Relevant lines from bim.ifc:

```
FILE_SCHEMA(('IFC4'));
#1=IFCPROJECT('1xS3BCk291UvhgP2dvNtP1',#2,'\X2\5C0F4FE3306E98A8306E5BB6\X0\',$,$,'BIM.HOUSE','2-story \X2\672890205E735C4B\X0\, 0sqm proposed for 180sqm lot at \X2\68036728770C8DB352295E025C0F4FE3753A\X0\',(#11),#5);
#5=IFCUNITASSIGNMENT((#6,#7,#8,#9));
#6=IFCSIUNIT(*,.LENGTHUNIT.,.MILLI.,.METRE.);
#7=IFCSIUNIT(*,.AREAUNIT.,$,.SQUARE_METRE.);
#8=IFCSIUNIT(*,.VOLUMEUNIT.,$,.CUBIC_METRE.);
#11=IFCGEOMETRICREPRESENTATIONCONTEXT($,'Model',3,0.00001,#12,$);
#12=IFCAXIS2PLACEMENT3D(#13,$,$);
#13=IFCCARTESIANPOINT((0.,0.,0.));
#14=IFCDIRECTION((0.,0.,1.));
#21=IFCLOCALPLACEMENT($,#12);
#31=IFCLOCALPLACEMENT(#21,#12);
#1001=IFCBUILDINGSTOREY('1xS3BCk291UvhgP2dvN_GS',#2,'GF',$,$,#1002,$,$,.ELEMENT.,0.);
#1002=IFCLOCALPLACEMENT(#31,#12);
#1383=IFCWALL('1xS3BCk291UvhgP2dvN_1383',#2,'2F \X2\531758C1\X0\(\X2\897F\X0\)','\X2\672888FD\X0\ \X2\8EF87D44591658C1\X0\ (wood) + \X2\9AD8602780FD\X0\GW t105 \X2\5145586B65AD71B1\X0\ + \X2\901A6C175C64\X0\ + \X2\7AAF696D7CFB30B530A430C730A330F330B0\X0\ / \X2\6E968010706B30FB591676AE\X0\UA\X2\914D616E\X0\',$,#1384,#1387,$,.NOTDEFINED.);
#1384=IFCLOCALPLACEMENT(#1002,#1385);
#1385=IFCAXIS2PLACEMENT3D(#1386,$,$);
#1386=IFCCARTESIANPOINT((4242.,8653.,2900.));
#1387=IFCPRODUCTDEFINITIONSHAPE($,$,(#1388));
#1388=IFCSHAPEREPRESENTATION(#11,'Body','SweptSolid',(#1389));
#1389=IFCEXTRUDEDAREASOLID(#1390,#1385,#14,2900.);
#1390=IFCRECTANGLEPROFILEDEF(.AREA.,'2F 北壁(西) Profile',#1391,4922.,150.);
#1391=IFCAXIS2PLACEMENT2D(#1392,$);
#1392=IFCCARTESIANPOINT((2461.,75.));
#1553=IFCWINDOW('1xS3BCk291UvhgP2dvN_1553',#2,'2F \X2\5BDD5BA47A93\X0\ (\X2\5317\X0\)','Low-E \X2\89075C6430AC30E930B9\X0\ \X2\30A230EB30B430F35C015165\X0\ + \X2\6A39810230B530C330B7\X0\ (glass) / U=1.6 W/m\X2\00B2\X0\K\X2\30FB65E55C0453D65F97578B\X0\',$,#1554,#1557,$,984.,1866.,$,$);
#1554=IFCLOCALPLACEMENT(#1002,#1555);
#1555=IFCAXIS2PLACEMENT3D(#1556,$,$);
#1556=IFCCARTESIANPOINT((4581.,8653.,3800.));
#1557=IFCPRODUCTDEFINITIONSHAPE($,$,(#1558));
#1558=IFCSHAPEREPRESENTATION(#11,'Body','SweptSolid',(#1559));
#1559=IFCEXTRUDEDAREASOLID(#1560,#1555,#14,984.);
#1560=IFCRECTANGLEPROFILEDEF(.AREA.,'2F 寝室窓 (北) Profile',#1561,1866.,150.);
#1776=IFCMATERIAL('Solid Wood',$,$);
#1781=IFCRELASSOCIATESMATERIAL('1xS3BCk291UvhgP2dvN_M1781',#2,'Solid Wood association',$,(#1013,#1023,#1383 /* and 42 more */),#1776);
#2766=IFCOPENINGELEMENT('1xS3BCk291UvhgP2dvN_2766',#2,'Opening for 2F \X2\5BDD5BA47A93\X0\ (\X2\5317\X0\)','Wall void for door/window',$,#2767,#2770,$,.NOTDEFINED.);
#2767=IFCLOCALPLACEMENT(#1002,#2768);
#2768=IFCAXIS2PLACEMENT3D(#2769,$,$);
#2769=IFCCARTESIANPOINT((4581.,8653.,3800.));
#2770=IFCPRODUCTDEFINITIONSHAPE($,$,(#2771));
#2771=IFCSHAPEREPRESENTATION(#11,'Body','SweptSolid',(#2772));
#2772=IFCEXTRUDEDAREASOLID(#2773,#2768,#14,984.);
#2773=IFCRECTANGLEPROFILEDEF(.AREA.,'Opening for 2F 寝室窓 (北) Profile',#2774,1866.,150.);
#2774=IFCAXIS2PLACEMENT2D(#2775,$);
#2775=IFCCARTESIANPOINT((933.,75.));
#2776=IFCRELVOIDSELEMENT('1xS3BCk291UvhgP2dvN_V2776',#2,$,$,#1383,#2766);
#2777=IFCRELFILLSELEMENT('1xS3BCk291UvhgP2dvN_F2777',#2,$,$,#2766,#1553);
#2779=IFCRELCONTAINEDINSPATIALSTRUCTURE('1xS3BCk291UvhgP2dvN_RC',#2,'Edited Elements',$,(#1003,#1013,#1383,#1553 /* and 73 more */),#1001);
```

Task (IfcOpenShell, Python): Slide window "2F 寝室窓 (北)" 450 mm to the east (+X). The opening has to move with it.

```python
import ifcopenshell
import ifcopenshell.api.geometry
import ifcopenshell.util.placement
import ifcopenshell.util.unit

model = ifcopenshell.open("bim.ifc")
unit_scale = ifcopenshell.util.unit.calculate_unit_scale(model)

window = model.by_guid("1xS3BCk291UvhgP2dvN_1553")
opening = window.FillsVoids[0].RelatingOpeningElement
wall = opening.VoidsElements[0].RelatingBuildingElement

wall_matrix = ifcopenshell.util.placement.get_local_placement(wall.ObjectPlacement)
shift = wall_matrix[:3, 0] * 0.45 / unit_scale
before = ifcopenshell.util.placement.get_local_placement(window.ObjectPlacement)[:3, 3].copy()

# The window is not placed relative to its opening, so move both.
for product in (opening, window):
    matrix = ifcopenshell.util.placement.get_local_placement(product.ObjectPlacement)
    matrix[:3, 3] += shift
    ifcopenshell.api.geometry.edit_object_placement(model, product=product, matrix=matrix, is_si=False)

after = ifcopenshell.util.placement.get_local_placement(window.ObjectPlacement)[:3, 3]
print("window moved by", (after - before).round(3) + 0.0)

model.write("bim-out.ifc")
```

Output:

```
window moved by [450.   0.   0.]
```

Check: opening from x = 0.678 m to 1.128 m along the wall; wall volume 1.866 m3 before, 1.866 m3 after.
